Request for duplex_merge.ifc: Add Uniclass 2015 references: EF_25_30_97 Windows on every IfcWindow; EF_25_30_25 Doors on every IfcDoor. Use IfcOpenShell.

First a look at what the model holds.

```python
import ifcopenshell

model = ifcopenshell.open("duplex_merge.ifc")
print(model.schema)
print("classifications:", [c.Name for c in model.by_type("IfcClassification")])
for ifc_class in ("IfcDoor", "IfcRoof", "IfcStair", "IfcWall", "IfcWindow"):
    print(ifc_class, len(model.by_type(ifc_class)))
```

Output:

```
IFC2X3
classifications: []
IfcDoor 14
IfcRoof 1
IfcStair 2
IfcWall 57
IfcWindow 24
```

```python
import ifcopenshell
import ifcopenshell.api.classification

model = ifcopenshell.open("duplex_merge.ifc")

# IFC2X3 requires Source and Edition and has no link from the project to the system.
system = model.create_entity("IfcClassification", Source="NBS", Edition="2015", Name="Uniclass 2015")

codes = {
    "IfcWindow": ("EF_25_30_97", "Windows"),
    "IfcDoor": ("EF_25_30_25", "Doors"),
}
for ifc_class, (code, name) in codes.items():
    products = model.by_type(ifc_class)
    ifcopenshell.api.classification.add_reference(
        model, products=products, classification=system, identification=code, name=name
    )
    print(code, len(products))

model.write("duplex_merge-out.ifc")
```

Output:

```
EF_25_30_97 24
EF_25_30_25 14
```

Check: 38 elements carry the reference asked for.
